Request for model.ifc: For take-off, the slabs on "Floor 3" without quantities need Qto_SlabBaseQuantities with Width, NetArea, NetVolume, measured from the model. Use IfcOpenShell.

First a look at what the model holds.

```python
import ifcopenshell
import ifcopenshell.util.element
import ifcopenshell.util.unit

model = ifcopenshell.open("model.ifc")
print(model.schema)
for unit_type in ("LENGTHUNIT", "AREAUNIT", "VOLUMEUNIT"):
    print(unit_type, ifcopenshell.util.unit.calculate_unit_scale(model, unit_type))
storey = next(s for s in model.by_type("IfcBuildingStorey") if s.Name == "Floor 3")
slabs = [e for e in ifcopenshell.util.element.get_decomposition(storey) if e.is_a("IfcSlab")]
for e in sorted(slabs, key=lambda e: e.id()):
    print(e.id(), e.is_a(), e.Name, list(ifcopenshell.util.element.get_psets(e, qtos_only=True)), sep=" | ")
```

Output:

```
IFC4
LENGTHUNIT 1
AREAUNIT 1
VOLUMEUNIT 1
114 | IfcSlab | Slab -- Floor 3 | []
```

```python
import ifcopenshell
import ifcopenshell.api.pset
import ifcopenshell.geom
import ifcopenshell.util.element
import ifcopenshell.util.shape
import ifcopenshell.util.unit

model = ifcopenshell.open("model.ifc")
unit_scale = ifcopenshell.util.unit.calculate_unit_scale(model)
area_scale = ifcopenshell.util.unit.calculate_unit_scale(model, "AREAUNIT")
volume_scale = ifcopenshell.util.unit.calculate_unit_scale(model, "VOLUMEUNIT")
settings = ifcopenshell.geom.settings()

storey = next(s for s in model.by_type("IfcBuildingStorey") if s.Name == "Floor 3")
slabs = [e for e in ifcopenshell.util.element.get_decomposition(storey) if e.is_a("IfcSlab")]

for e in sorted(slabs, key=lambda e: e.id()):
    if ifcopenshell.util.element.get_psets(e, qtos_only=True, should_inherit=False):
        continue
    # Geometry comes back in metres, in the element's own axes.
    shape = ifcopenshell.geom.create_shape(settings, e)
    values = {
        "Width": ifcopenshell.util.shape.get_z(shape.geometry) / unit_scale,
        "NetArea": ifcopenshell.util.shape.get_footprint_area(shape.geometry) / area_scale,
        "NetVolume": ifcopenshell.util.shape.get_volume(shape.geometry) / volume_scale,
    }
    qto = ifcopenshell.api.pset.add_qto(model, product=e, name="Qto_SlabBaseQuantities")
    ifcopenshell.api.pset.edit_qto(model, qto=qto, properties=values)
    print(e.id(), {k: round(v, 3) for k, v in values.items()})

model.write("model_edited.ifc")
```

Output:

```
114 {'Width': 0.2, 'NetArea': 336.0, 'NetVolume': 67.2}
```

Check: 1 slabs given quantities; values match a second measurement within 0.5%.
